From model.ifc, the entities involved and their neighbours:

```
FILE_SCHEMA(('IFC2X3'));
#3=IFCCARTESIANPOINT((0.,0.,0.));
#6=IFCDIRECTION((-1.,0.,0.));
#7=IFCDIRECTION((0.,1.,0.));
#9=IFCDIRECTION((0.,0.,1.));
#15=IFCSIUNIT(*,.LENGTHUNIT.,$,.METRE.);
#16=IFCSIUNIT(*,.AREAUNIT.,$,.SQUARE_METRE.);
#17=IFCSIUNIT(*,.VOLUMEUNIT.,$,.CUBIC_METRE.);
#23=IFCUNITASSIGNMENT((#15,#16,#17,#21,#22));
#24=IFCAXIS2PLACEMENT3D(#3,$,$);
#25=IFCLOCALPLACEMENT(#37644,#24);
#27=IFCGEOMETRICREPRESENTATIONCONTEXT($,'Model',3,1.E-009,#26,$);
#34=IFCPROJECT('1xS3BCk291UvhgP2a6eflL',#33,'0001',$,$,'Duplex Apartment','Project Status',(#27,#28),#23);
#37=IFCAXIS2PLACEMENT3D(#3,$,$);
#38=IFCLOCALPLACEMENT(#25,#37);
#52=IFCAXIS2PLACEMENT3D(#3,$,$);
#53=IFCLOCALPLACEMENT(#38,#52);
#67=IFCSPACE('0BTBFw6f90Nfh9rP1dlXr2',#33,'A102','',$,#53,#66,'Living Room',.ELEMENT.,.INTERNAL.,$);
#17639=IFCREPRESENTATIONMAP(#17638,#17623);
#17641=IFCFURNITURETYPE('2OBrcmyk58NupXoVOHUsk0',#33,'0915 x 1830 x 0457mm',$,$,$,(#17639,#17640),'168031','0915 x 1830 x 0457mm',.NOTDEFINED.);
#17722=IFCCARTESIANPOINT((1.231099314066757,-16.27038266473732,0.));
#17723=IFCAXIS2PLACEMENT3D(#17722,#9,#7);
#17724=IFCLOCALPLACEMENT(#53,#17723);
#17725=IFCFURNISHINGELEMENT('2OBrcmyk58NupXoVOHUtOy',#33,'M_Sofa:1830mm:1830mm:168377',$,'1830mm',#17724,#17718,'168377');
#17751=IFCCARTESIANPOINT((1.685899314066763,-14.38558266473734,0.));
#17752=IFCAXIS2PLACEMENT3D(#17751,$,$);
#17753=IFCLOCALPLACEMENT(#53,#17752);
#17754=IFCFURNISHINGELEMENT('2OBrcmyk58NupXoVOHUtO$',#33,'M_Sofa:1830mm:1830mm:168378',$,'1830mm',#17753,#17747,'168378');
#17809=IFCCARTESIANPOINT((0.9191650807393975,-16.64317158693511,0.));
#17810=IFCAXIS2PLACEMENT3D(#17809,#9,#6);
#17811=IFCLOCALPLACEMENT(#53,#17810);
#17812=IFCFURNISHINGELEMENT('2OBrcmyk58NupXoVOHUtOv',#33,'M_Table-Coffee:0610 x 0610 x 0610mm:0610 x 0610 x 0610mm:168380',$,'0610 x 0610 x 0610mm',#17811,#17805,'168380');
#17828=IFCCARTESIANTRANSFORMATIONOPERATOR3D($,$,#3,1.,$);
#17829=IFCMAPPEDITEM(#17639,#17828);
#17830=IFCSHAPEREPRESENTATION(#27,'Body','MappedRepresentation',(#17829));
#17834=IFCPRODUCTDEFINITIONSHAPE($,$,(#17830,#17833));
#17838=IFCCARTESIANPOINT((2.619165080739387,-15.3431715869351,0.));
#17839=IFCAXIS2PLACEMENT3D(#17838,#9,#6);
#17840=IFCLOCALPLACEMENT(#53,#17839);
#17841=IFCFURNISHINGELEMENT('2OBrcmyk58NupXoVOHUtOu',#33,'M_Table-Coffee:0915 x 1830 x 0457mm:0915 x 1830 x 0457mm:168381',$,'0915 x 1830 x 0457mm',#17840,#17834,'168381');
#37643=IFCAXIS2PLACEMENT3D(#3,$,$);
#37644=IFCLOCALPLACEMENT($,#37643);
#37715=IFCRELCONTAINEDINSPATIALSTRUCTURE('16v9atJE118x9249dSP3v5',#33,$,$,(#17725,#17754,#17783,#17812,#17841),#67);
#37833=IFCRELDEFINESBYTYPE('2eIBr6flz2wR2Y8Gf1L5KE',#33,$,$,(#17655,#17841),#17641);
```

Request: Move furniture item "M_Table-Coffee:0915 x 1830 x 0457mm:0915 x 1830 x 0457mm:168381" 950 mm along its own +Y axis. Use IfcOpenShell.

```python
import ifcopenshell
import ifcopenshell.api.geometry
import ifcopenshell.util.placement

model = ifcopenshell.open("model.ifc")

item = model.by_guid("2OBrcmyk58NupXoVOHUtOu")
matrix = ifcopenshell.util.placement.get_local_placement(item.ObjectPlacement)
matrix[:3, 3] += matrix[:3, 1] * 0.95
ifcopenshell.api.geometry.edit_object_placement(model, product=item, matrix=matrix, is_si=False)

print(ifcopenshell.util.placement.get_local_placement(item.ObjectPlacement).round(3) + 0.0)

model.write("model_rev.ifc")
```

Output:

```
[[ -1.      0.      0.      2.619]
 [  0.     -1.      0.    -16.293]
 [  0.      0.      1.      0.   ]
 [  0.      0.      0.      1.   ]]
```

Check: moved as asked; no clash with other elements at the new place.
